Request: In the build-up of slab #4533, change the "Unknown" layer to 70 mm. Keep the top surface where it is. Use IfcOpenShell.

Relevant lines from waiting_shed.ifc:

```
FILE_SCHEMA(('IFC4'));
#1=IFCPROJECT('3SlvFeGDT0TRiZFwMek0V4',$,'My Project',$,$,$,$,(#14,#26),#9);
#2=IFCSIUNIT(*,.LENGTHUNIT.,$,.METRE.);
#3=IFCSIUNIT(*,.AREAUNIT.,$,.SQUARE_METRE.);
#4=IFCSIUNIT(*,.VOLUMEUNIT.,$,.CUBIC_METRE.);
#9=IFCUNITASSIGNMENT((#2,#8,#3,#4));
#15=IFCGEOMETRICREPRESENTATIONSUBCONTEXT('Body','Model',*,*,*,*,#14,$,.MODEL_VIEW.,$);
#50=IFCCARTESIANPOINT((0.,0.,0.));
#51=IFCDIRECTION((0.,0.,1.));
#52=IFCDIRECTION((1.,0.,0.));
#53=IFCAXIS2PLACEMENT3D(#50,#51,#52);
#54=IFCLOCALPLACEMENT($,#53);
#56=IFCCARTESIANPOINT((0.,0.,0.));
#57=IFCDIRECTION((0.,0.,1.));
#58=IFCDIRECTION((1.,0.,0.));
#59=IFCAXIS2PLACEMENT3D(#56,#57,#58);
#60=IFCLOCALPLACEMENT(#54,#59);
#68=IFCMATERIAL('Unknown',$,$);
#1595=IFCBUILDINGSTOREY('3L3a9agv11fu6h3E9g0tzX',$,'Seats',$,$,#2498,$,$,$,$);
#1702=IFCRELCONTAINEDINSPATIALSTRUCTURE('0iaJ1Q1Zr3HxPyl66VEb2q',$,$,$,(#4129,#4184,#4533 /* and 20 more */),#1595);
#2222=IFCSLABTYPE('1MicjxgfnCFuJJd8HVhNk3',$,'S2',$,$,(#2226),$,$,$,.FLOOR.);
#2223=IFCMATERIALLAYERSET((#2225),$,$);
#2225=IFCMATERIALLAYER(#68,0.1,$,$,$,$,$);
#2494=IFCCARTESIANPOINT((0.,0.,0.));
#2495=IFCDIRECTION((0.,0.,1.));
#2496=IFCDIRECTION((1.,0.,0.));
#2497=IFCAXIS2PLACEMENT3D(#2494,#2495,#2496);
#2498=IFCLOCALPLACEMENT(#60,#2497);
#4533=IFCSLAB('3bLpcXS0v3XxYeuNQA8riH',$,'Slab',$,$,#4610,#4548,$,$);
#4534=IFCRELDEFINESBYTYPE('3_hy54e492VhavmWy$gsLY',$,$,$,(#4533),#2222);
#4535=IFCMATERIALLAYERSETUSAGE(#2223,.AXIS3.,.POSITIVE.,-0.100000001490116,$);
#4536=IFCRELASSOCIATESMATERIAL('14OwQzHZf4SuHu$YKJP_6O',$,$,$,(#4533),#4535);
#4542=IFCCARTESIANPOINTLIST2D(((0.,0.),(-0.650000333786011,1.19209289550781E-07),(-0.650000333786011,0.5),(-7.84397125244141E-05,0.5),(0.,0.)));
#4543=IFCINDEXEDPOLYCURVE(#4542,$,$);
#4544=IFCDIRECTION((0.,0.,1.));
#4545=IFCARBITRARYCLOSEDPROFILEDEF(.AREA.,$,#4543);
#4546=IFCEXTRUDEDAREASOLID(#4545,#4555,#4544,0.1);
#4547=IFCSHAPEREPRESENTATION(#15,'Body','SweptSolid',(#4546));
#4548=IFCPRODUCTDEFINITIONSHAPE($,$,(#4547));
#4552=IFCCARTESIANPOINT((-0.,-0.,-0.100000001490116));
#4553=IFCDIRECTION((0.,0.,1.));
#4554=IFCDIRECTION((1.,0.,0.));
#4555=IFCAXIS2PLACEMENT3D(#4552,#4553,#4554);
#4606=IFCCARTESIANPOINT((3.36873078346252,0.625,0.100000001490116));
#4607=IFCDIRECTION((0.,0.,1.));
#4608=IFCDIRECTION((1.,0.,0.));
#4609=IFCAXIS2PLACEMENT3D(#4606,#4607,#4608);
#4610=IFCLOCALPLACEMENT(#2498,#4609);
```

```python
import ifcopenshell
import ifcopenshell.util.element
import ifcopenshell.util.representation

model = ifcopenshell.open("waiting_shed.ifc")

layer_set = model.by_id(2223)
layer = next(l for l in layer_set.MaterialLayers if l.Material and l.Material.Name == "Unknown")
change = 0.07 - layer.LayerThickness
layer.LayerThickness += change

# Geometry does not follow the layer set by itself.
slabs = [e for e in ifcopenshell.util.element.get_elements_by_material(model, layer_set) if e.is_a("IfcSlab")]
for slab in sorted(slabs, key=lambda e: e.id()):
    body = ifcopenshell.util.representation.get_representation(slab, "Model", "Body")
    solid = body.Items[0]
    old_depth = solid.Depth
    solid.Depth += change
    # Extruded upwards: lower the start of the extrusion so the top stays.
    x, y, z = solid.Position.Location.Coordinates
    solid.Position.Location = model.createIfcCartesianPoint((x, y, z - change))
    print(slab.id(), f"{old_depth:g} -> {solid.Depth:g}")

# The layers are counted up from the underside, which has moved.
for usage in {ifcopenshell.util.element.get_material(slab) for slab in slabs}:
    usage.OffsetFromReferenceLine -= change

model.write("waiting_shed_v2.ifc")
```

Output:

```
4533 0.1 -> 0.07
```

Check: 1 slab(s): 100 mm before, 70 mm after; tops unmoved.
